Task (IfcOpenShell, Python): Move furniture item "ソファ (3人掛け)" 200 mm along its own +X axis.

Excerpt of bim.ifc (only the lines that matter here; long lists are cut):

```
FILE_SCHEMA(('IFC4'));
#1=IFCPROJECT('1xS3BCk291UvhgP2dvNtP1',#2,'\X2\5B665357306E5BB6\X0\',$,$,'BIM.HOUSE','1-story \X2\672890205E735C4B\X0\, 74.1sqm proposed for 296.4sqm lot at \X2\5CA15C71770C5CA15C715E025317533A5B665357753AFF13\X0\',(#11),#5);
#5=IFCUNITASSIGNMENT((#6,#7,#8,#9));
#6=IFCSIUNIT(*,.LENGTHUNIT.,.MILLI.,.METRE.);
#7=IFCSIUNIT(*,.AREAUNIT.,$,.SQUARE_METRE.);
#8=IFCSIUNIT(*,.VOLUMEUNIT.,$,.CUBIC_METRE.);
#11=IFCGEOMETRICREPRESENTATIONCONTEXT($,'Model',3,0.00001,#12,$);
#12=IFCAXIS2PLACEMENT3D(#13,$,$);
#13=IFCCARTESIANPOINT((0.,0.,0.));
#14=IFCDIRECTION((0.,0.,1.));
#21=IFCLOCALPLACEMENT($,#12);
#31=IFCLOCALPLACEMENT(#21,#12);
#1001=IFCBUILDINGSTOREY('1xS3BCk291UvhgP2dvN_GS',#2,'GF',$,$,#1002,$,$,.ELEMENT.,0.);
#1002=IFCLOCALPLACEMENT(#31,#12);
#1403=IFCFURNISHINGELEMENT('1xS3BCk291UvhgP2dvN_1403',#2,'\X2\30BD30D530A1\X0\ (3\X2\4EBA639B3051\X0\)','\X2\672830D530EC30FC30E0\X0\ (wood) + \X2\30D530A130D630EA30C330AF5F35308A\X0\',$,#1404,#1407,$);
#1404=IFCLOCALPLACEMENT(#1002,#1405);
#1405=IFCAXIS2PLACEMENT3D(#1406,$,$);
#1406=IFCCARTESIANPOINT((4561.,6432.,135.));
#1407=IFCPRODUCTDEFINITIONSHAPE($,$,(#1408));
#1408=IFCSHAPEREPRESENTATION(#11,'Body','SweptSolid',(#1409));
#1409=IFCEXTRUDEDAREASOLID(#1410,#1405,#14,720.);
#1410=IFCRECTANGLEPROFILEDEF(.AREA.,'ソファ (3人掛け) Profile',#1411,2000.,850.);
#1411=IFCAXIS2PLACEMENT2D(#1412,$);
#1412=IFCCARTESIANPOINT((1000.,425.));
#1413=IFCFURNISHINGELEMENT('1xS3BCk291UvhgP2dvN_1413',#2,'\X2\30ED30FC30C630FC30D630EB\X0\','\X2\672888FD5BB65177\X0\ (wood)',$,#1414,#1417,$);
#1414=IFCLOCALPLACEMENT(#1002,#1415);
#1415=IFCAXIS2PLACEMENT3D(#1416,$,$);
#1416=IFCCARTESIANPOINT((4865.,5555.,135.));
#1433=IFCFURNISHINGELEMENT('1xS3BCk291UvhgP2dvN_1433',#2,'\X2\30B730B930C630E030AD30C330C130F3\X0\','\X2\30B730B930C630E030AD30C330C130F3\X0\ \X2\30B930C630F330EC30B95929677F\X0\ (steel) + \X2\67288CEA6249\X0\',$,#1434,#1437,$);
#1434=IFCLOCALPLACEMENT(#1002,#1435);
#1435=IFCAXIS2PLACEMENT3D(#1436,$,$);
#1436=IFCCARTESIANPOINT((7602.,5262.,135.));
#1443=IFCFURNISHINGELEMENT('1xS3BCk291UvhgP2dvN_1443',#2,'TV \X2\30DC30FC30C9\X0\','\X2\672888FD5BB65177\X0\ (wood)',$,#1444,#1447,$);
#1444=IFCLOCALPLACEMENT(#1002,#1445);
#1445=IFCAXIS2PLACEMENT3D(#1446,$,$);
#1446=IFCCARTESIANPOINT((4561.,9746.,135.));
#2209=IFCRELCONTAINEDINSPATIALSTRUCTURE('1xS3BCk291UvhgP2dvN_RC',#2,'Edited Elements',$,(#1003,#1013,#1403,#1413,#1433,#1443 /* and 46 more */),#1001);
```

```python
import ifcopenshell
import ifcopenshell.api.geometry
import ifcopenshell.util.placement
import ifcopenshell.util.unit

model = ifcopenshell.open("bim.ifc")
unit_scale = ifcopenshell.util.unit.calculate_unit_scale(model)

item = model.by_id(1403)
matrix = ifcopenshell.util.placement.get_local_placement(item.ObjectPlacement)
matrix[:3, 3] += matrix[:3, 0] * 0.2 / unit_scale
ifcopenshell.api.geometry.edit_object_placement(model, product=item, matrix=matrix, is_si=False)

print(ifcopenshell.util.placement.get_local_placement(item.ObjectPlacement).round(3) + 0.0)

model.write("bim_v2.ifc")
```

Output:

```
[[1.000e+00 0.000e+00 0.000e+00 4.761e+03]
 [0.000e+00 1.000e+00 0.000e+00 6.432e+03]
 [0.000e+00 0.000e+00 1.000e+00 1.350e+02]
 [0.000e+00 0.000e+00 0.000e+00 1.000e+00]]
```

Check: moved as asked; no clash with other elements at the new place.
